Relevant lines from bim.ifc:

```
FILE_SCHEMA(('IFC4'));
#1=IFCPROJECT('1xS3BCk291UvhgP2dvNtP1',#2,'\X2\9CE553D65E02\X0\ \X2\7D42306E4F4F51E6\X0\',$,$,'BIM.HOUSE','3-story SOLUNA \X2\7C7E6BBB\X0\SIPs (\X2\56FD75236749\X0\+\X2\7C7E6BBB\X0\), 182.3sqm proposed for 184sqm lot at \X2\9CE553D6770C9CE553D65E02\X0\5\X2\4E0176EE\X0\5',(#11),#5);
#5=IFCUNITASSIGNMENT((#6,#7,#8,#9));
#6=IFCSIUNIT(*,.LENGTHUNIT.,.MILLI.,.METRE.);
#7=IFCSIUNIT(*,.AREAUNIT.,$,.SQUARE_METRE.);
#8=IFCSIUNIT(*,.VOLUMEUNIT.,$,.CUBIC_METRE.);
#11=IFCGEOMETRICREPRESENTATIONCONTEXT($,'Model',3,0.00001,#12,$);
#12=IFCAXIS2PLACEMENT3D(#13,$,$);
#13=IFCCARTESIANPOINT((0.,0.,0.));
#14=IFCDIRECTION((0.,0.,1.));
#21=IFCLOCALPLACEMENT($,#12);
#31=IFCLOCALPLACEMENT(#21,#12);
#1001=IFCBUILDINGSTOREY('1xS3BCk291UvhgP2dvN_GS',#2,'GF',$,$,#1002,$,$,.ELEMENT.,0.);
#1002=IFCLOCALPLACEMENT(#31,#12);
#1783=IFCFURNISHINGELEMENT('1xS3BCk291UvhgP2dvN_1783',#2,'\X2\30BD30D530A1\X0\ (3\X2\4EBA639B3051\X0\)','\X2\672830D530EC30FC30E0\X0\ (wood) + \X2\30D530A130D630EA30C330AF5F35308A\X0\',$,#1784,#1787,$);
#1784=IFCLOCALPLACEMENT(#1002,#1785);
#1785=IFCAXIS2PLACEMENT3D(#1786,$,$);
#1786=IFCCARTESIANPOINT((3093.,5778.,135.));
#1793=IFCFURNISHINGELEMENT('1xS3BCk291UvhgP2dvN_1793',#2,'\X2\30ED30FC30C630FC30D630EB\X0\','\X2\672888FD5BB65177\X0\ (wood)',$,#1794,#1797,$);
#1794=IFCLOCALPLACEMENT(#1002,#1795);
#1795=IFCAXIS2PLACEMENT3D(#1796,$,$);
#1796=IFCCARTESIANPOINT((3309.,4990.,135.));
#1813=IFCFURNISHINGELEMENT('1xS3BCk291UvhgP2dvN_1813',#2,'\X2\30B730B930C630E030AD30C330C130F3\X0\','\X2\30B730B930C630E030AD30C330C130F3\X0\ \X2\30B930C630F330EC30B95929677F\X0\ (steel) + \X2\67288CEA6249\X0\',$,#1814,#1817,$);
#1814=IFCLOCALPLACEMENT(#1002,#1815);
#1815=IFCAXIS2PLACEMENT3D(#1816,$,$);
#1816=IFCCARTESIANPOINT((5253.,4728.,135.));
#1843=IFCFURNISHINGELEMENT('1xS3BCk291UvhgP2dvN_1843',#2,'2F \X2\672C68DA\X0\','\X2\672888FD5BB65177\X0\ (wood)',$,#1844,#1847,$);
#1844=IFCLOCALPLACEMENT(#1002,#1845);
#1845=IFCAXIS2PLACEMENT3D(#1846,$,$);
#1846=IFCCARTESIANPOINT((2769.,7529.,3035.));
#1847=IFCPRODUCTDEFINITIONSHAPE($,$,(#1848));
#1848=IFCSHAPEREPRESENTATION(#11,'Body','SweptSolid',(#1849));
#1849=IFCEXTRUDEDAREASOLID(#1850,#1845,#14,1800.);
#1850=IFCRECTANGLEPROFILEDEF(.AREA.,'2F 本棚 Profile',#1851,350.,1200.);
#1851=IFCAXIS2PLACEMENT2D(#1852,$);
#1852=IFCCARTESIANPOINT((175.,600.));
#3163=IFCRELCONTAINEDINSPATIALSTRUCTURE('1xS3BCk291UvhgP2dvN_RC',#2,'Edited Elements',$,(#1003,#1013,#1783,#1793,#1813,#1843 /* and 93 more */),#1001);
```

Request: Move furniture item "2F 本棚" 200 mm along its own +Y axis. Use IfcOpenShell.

```python
import ifcopenshell
import ifcopenshell.api.geometry
import ifcopenshell.util.placement
import ifcopenshell.util.unit

model = ifcopenshell.open("bim.ifc")
unit_scale = ifcopenshell.util.unit.calculate_unit_scale(model)

item = model.by_guid("1xS3BCk291UvhgP2dvN_1843")
matrix = ifcopenshell.util.placement.get_local_placement(item.ObjectPlacement)
matrix[:3, 3] += matrix[:3, 1] * 0.2 / unit_scale
ifcopenshell.api.geometry.edit_object_placement(model, product=item, matrix=matrix, is_si=False)

print(ifcopenshell.util.placement.get_local_placement(item.ObjectPlacement).round(3) + 0.0)

model.write("bim_v2.ifc")
```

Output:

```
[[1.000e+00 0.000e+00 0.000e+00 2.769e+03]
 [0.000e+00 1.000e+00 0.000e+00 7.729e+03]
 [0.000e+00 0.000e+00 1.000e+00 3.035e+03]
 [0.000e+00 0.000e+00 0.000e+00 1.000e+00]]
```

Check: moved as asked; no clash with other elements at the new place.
